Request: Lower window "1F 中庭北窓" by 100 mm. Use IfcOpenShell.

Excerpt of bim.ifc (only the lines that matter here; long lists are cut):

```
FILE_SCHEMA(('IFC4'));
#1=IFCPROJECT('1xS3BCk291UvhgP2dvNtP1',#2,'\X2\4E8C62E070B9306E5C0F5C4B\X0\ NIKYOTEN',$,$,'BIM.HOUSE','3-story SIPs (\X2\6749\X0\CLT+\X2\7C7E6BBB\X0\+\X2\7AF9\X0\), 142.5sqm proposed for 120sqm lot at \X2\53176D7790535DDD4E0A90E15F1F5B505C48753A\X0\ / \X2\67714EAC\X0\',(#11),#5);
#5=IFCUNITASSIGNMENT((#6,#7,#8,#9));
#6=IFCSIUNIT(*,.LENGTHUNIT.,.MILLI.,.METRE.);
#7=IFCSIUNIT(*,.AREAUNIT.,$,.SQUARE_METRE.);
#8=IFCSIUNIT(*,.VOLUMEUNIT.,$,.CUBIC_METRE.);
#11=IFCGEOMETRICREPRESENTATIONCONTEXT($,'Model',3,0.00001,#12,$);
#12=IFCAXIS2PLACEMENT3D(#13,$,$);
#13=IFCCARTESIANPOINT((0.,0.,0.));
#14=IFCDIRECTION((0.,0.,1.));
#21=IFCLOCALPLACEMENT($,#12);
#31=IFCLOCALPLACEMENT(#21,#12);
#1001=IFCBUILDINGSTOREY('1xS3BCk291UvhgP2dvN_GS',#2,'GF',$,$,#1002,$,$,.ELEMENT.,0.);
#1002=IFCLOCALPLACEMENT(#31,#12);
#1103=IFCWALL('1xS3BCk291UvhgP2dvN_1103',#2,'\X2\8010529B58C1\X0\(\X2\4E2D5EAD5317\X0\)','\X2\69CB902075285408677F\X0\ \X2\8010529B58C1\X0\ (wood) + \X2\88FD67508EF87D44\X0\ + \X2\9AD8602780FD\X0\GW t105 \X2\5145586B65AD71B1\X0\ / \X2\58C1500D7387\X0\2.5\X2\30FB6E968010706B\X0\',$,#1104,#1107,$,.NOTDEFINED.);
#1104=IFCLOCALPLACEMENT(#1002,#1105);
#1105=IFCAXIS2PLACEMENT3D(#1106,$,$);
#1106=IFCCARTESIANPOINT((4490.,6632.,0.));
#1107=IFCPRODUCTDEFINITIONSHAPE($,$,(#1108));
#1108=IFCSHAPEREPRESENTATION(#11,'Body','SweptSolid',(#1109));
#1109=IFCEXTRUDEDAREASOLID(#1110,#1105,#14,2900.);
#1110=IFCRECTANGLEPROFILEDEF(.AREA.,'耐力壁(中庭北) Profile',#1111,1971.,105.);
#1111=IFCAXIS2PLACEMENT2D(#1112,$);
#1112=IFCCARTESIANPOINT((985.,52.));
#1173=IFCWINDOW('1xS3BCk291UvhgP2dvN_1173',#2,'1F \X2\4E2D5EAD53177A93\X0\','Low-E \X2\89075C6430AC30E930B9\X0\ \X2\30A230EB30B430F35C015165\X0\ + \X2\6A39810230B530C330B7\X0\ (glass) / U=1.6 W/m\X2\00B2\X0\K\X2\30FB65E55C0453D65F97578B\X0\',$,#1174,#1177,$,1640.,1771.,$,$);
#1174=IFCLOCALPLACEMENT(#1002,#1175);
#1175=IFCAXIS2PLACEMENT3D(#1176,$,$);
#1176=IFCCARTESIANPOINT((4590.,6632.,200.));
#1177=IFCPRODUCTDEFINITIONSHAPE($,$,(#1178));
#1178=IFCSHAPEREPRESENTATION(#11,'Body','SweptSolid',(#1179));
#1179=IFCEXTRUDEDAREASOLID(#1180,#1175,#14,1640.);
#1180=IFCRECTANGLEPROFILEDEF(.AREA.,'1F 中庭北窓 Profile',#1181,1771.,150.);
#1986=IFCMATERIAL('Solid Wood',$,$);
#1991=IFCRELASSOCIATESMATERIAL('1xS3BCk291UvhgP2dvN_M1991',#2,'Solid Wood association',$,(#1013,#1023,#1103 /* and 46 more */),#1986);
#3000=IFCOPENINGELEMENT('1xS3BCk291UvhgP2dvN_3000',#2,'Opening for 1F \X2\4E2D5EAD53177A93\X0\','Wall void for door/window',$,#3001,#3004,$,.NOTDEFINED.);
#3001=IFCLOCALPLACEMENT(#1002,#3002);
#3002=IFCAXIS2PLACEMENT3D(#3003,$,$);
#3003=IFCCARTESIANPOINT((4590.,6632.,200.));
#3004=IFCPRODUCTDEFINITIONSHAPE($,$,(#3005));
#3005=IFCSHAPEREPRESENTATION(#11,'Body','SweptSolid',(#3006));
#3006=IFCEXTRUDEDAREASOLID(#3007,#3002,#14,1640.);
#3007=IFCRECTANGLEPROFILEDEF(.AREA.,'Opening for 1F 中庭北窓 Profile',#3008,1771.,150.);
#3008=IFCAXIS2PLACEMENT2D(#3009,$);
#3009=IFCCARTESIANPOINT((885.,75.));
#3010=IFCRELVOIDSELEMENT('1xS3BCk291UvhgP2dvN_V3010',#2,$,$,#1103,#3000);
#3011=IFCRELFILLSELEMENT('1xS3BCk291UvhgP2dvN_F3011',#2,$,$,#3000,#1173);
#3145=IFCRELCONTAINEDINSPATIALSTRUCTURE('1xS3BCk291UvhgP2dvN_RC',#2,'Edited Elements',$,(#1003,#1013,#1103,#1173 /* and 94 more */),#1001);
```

```python
import numpy as np
import ifcopenshell
import ifcopenshell.api.geometry
import ifcopenshell.util.placement
import ifcopenshell.util.unit

model = ifcopenshell.open("bim.ifc")
unit_scale = ifcopenshell.util.unit.calculate_unit_scale(model)

window = model.by_guid("1xS3BCk291UvhgP2dvN_1173")
opening = window.FillsVoids[0].RelatingOpeningElement
dz = -100.0

shift = np.array([0.0, 0.0, dz])
# The window is not placed relative to its opening, so move both.
for product in (opening, window):
    matrix = ifcopenshell.util.placement.get_local_placement(product.ObjectPlacement)
    matrix[:3, 3] += shift
    ifcopenshell.api.geometry.edit_object_placement(model, product=product, matrix=matrix, is_si=False)

print(f"moved by {dz * unit_scale:+.3f} m")

model.write("bim_updated.ifc")
```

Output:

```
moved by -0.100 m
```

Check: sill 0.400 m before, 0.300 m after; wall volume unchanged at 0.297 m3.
